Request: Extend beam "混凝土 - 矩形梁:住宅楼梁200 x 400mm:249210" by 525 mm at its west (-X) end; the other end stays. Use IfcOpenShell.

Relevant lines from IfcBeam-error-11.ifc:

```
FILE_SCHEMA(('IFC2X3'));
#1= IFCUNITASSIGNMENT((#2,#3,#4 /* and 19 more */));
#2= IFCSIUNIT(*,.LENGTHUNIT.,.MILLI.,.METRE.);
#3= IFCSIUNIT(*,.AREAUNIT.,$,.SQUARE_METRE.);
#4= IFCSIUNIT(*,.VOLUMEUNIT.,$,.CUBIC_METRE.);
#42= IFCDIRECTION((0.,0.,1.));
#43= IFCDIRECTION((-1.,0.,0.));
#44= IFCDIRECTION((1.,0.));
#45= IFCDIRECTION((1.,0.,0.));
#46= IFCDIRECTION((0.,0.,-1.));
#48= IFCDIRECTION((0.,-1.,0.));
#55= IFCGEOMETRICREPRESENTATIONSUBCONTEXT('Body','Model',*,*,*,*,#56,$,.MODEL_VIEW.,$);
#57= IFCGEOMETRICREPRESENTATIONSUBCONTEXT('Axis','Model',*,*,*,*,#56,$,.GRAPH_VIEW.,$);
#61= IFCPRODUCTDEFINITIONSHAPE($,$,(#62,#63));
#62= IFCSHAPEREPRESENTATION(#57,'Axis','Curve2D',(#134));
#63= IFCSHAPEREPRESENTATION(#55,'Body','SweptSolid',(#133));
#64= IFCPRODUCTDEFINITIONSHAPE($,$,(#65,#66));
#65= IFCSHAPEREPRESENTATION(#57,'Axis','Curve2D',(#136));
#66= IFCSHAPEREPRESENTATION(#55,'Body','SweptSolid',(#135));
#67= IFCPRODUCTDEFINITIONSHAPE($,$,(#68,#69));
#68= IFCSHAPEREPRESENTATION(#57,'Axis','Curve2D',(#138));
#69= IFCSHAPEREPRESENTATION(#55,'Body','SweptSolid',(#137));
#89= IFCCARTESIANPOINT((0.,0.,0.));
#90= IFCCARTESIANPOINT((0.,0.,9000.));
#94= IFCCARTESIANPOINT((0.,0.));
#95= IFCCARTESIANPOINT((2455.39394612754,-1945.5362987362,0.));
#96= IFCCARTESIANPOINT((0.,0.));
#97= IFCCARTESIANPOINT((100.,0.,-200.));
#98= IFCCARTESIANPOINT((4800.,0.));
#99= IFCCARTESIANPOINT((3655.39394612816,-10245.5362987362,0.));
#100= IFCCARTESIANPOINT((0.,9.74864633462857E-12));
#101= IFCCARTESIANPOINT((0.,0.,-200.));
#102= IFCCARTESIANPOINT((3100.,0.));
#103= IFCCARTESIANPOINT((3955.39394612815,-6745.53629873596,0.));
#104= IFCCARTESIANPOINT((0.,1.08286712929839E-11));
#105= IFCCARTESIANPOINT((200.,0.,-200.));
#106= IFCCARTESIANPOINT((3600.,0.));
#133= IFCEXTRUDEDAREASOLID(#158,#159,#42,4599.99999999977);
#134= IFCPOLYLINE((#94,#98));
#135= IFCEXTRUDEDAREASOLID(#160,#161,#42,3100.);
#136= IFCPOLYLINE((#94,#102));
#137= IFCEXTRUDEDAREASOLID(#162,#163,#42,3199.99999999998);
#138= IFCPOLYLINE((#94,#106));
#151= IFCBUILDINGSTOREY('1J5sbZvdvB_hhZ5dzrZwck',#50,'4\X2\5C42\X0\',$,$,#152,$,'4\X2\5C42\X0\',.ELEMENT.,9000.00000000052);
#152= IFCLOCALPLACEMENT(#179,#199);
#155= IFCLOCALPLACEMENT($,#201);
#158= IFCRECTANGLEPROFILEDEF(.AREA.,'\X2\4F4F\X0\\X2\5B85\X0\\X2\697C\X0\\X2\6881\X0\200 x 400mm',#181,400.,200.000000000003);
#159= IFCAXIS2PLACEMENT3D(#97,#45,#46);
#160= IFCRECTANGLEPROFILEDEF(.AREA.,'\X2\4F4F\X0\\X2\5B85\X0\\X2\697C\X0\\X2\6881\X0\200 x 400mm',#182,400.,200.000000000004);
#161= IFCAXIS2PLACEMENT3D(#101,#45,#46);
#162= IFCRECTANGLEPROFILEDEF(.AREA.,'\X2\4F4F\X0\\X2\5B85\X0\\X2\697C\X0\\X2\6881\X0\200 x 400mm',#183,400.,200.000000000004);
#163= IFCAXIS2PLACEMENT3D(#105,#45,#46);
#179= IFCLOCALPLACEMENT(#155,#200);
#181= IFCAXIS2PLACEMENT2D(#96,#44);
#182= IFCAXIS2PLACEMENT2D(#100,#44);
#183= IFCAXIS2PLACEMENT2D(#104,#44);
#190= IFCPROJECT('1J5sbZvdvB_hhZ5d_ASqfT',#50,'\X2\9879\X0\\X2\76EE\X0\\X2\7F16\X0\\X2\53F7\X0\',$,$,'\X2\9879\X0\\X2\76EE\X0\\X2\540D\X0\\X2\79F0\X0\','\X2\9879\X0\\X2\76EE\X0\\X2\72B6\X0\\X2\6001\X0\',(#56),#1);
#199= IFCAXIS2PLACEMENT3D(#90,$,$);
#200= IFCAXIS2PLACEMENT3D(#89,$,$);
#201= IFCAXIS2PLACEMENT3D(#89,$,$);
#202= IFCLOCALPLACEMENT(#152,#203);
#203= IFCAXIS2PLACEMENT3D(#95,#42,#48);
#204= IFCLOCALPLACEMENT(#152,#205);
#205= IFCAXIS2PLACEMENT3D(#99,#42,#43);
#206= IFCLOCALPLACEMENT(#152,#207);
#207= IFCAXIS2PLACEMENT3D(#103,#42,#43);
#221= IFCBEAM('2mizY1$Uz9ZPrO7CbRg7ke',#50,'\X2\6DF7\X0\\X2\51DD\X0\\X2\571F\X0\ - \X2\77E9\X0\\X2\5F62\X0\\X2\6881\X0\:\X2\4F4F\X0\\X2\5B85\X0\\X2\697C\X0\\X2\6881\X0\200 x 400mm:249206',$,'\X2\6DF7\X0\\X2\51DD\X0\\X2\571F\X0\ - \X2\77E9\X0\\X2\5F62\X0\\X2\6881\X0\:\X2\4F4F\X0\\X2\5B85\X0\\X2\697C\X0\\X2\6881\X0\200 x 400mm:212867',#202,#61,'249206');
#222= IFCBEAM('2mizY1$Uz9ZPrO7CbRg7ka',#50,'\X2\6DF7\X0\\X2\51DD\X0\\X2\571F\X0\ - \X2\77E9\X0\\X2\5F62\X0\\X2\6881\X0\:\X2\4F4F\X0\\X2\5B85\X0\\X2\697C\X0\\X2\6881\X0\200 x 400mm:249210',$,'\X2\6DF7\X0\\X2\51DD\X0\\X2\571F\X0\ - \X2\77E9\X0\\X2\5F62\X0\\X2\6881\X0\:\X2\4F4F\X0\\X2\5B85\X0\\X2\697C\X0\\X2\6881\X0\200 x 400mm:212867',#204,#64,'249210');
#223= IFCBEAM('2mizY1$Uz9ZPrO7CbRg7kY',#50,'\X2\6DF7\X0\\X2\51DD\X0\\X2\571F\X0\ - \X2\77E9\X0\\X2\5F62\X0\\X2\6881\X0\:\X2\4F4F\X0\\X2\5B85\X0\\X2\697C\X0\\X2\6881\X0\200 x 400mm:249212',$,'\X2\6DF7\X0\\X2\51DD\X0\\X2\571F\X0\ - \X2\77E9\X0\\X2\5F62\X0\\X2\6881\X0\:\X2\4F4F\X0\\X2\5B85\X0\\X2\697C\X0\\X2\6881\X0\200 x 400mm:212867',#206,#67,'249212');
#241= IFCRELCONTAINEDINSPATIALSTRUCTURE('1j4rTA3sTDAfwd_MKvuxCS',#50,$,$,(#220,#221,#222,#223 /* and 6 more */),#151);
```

```python
import numpy as np
import ifcopenshell
import ifcopenshell.util.representation

model = ifcopenshell.open("IfcBeam-error-11.ifc")

member = model.by_guid("2mizY1$Uz9ZPrO7CbRg7ka")
change = 525.0

# The extrusion runs towards the end named, so only its depth changes.
body = ifcopenshell.util.representation.get_representation(member, "Model", "Body")
solid = body.Items[0]
old_length = solid.Depth
solid.Depth += change

# Move the axis end point with it.
axis = next(r for r in member.Representation.Representations if r.RepresentationIdentifier == "Axis").Items[0]
start, end = (np.array(p.Coordinates) for p in axis.Points)
end = end + (end - start) / np.linalg.norm(end - start) * change
point = model.createIfcCartesianPoint(end.tolist())
axis.Points = [axis.Points[0], point]

print(f"length {old_length:g} -> {solid.Depth:g}")

model.write("IfcBeam-error-11-out.ifc")
```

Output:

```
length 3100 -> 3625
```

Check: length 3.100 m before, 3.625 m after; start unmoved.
